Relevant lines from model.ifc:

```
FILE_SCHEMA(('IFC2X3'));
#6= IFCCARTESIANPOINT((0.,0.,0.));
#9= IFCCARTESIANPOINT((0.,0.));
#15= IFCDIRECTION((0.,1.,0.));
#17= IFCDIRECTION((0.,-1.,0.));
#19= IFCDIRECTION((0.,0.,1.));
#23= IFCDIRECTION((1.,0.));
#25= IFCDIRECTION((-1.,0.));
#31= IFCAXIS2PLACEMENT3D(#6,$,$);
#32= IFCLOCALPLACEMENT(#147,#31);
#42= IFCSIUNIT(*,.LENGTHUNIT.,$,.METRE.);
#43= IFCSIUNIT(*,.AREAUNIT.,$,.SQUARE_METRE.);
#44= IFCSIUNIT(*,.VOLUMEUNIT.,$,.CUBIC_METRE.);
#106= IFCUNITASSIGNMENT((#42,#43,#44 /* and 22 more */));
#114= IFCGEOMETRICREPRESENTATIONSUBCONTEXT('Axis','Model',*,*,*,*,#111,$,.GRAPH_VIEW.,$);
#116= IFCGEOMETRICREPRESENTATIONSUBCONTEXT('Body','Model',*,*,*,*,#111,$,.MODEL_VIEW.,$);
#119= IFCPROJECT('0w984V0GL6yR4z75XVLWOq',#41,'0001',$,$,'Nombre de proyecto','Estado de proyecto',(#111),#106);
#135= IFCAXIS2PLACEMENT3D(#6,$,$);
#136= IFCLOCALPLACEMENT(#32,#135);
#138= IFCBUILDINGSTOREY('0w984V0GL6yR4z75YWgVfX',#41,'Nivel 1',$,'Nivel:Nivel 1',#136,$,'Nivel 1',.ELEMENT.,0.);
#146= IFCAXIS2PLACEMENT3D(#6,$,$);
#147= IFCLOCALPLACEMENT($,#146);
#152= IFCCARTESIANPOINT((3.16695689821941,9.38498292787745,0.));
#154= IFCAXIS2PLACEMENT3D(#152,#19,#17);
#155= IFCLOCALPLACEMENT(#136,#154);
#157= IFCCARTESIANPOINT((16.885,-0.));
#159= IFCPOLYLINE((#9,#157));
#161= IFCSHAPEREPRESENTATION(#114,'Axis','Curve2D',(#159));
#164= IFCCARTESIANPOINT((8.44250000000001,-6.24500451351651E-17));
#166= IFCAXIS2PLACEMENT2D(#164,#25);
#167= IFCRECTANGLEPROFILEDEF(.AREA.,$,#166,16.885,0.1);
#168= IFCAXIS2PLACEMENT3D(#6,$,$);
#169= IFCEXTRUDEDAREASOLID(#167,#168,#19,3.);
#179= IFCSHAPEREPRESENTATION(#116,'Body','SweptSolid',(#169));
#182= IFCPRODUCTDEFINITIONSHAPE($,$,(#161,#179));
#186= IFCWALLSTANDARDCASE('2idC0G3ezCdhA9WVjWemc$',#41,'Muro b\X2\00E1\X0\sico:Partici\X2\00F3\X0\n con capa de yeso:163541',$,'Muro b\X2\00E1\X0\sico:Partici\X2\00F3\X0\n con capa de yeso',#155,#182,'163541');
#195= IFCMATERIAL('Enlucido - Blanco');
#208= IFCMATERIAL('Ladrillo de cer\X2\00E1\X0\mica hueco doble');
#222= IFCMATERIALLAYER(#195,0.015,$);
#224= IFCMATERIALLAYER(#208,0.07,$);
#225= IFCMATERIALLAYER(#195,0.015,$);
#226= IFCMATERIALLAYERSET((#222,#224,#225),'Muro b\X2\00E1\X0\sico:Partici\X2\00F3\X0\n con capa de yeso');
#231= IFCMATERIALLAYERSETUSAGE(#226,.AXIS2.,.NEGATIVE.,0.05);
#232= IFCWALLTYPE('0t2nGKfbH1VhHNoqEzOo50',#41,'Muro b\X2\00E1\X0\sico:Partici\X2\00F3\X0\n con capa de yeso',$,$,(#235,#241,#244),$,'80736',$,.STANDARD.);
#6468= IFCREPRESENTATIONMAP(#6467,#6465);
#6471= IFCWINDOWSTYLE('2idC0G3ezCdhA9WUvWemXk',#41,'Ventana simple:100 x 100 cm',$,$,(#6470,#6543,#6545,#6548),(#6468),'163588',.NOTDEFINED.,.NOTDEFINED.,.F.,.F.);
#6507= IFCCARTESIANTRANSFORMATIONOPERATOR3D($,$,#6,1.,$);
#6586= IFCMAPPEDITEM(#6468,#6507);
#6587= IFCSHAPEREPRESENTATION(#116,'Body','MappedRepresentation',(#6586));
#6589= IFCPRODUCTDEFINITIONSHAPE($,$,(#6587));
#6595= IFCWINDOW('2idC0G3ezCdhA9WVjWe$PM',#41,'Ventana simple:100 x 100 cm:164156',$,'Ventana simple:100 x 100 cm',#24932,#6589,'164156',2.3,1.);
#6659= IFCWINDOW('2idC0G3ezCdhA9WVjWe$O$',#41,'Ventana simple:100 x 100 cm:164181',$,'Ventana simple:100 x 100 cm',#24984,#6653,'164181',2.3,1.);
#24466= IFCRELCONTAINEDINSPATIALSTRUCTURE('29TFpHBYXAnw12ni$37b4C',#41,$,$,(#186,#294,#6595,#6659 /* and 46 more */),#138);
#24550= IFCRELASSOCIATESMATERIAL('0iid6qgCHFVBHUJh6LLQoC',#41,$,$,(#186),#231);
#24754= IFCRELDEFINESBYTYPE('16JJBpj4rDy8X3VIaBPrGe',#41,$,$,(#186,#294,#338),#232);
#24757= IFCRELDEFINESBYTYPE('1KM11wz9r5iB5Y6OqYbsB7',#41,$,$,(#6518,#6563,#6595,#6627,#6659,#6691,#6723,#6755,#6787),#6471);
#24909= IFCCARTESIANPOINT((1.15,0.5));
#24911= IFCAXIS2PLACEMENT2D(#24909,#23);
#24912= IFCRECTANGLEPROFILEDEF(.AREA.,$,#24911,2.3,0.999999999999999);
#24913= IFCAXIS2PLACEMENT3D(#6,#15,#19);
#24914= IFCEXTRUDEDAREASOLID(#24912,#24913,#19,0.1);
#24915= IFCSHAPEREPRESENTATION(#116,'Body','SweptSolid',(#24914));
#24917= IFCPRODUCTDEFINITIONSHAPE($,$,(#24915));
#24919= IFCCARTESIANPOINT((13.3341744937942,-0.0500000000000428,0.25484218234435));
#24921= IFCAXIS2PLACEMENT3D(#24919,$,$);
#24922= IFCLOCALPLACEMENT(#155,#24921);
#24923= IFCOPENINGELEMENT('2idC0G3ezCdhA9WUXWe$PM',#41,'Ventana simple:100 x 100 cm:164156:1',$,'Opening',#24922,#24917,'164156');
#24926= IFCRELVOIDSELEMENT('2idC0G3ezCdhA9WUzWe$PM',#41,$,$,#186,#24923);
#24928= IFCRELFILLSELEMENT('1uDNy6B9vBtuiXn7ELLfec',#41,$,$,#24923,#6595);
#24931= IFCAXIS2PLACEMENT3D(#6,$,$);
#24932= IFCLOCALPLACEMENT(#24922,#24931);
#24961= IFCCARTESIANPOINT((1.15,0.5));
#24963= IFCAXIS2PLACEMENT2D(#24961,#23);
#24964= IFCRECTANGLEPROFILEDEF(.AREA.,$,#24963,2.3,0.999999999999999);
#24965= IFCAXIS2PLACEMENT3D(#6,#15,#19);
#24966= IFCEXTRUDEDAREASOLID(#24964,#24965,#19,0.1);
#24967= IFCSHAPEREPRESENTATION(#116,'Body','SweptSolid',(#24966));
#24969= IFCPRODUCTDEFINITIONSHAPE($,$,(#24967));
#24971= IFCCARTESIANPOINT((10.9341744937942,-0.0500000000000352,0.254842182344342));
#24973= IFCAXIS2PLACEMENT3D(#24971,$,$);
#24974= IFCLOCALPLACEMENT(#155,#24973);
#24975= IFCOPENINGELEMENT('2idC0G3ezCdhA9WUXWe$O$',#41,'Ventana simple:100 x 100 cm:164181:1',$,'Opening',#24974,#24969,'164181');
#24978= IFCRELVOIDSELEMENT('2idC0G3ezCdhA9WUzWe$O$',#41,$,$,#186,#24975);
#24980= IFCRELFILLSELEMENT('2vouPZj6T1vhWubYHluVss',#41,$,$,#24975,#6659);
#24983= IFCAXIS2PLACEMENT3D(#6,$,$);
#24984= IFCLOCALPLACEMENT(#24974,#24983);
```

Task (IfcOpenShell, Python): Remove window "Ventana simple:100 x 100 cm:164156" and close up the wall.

```python
import ifcopenshell
import ifcopenshell.api.feature
import ifcopenshell.api.root
import ifcopenshell.geom
import ifcopenshell.util.shape

model = ifcopenshell.open("model.ifc")
settings = ifcopenshell.geom.settings()


def volume(element):
    """Net volume in cubic metres, openings subtracted."""
    shape = ifcopenshell.geom.create_shape(settings, element)
    return ifcopenshell.util.shape.get_volume(shape.geometry)


window = model.by_id(6595)
opening = window.FillsVoids[0].RelatingOpeningElement
wall = opening.VoidsElements[0].RelatingBuildingElement
before = volume(wall)

ifcopenshell.api.root.remove_product(model, product=window)
ifcopenshell.api.feature.remove_feature(model, feature=opening)

after = volume(wall)

print(f"wall volume {before:.3f} -> {after:.3f} m3")

model.write("model-out.ifc")
```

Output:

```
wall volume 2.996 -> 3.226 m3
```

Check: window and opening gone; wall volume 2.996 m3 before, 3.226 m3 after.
